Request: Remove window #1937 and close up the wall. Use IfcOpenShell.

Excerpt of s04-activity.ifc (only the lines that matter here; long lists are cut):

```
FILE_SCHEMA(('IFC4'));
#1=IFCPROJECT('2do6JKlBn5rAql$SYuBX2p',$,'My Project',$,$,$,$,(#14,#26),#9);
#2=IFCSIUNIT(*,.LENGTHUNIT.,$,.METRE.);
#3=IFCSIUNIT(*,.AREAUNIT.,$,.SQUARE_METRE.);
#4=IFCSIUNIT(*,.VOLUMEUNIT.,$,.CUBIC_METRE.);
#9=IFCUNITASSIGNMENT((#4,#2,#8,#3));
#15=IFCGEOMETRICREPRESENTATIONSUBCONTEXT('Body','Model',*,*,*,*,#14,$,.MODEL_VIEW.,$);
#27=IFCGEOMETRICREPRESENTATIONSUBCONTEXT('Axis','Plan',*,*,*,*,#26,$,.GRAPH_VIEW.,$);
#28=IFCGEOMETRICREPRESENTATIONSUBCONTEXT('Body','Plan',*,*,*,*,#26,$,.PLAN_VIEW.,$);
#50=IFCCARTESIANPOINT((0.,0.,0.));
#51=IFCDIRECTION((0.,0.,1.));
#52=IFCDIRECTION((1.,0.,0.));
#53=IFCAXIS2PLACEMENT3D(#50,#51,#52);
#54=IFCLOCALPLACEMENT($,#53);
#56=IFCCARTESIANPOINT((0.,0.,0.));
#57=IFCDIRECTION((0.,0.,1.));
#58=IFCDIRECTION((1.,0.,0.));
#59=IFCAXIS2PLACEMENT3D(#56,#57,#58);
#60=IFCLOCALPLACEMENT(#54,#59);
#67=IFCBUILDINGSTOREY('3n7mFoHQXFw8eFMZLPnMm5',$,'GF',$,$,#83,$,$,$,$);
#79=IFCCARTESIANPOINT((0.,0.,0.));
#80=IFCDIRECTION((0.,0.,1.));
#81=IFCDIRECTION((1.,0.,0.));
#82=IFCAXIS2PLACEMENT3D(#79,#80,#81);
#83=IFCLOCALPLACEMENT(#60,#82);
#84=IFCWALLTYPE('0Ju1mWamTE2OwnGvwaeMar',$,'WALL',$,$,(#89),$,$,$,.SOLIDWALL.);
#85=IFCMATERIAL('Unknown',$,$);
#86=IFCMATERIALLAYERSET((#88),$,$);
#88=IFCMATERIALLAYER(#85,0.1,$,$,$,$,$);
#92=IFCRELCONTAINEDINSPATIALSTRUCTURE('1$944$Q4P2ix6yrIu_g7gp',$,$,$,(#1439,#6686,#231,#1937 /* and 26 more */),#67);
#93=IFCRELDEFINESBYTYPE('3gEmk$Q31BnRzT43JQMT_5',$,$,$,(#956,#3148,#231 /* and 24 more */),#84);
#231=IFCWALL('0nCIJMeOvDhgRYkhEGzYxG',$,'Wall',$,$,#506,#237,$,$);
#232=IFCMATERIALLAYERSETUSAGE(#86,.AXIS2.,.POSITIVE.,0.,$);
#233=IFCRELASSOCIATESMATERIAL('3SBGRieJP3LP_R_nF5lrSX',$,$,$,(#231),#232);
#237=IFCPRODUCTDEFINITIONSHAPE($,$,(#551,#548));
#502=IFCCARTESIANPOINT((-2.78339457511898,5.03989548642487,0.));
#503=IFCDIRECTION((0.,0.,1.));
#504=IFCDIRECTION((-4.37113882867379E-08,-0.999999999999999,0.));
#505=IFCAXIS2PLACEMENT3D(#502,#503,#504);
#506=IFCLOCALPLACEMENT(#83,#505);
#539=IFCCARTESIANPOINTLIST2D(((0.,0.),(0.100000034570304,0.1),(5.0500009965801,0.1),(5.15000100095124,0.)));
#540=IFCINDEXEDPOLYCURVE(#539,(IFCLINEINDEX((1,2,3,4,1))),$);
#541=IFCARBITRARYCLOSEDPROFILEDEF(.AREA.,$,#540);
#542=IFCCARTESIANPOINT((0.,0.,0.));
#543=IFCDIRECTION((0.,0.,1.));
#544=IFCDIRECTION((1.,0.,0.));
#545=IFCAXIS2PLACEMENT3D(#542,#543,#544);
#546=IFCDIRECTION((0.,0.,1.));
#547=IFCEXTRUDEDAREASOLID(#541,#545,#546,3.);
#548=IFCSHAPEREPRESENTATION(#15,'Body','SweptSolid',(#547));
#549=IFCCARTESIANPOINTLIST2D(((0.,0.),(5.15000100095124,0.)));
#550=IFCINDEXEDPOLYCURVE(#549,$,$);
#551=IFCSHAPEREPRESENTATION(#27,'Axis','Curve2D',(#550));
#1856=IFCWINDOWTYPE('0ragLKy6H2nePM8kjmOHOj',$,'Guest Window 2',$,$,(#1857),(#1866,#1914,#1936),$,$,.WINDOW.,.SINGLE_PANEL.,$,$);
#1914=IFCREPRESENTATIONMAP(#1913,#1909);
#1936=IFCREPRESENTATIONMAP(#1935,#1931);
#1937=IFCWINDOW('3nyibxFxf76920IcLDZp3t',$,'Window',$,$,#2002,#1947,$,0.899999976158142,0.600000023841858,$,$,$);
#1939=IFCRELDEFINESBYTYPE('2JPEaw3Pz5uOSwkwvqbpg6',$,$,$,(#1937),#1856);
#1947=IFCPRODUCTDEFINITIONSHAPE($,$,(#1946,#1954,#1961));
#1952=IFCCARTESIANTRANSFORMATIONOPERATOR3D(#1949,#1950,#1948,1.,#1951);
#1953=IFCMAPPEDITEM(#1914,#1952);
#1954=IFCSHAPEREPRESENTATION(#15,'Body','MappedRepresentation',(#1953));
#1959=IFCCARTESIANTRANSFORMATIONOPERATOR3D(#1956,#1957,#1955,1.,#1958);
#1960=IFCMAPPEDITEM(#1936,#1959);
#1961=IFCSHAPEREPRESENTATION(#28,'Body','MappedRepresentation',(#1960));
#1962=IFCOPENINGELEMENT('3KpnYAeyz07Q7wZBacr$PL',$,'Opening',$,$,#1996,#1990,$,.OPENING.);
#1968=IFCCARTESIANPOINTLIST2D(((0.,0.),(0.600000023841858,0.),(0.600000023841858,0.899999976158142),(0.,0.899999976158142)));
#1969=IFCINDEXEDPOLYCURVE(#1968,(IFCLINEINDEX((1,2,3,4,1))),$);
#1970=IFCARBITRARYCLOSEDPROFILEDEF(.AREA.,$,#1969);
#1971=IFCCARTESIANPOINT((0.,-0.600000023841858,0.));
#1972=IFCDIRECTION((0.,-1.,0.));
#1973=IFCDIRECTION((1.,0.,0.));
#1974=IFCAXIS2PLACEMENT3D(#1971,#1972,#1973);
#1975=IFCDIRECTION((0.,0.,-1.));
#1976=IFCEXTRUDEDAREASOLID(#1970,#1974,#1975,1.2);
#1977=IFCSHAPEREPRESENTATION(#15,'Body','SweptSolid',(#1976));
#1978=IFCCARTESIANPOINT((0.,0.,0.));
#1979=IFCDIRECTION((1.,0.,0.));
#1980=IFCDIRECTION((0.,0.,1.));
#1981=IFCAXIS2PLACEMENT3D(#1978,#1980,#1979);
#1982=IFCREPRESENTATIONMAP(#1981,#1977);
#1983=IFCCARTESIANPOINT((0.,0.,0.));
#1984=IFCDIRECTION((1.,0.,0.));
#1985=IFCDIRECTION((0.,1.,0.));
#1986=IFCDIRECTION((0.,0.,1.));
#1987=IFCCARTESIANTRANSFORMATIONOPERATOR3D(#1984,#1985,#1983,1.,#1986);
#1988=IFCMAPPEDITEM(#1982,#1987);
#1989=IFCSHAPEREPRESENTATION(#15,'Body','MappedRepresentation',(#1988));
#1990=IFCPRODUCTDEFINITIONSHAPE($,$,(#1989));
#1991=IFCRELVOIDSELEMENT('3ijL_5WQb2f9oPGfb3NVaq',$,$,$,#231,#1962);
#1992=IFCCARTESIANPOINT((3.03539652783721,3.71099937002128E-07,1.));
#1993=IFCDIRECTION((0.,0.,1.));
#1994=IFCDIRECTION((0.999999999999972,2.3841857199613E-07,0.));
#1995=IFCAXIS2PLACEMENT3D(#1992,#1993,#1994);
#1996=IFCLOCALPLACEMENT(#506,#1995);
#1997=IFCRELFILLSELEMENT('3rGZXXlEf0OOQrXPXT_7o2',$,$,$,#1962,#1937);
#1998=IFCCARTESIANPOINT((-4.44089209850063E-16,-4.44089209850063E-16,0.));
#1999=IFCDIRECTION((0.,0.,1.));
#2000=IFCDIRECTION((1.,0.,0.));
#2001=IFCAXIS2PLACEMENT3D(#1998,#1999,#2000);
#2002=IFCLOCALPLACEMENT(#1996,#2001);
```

```python
import ifcopenshell
import ifcopenshell.api.feature
import ifcopenshell.api.root
import ifcopenshell.geom
import ifcopenshell.util.shape

model = ifcopenshell.open("s04-activity.ifc")
settings = ifcopenshell.geom.settings()


def volume(element):
    """Net volume in cubic metres, openings subtracted."""
    shape = ifcopenshell.geom.create_shape(settings, element)
    return ifcopenshell.util.shape.get_volume(shape.geometry)


window = model.by_guid("3nyibxFxf76920IcLDZp3t")
opening = window.FillsVoids[0].RelatingOpeningElement
wall = opening.VoidsElements[0].RelatingBuildingElement
before = volume(wall)

ifcopenshell.api.root.remove_product(model, product=window)
ifcopenshell.api.feature.remove_feature(model, feature=opening)

after = volume(wall)

print(f"wall volume {before:.3f} -> {after:.3f} m3")

model.write("s04-activity_edited.ifc")
```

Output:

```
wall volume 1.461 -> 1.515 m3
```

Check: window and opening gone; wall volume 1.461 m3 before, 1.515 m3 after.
